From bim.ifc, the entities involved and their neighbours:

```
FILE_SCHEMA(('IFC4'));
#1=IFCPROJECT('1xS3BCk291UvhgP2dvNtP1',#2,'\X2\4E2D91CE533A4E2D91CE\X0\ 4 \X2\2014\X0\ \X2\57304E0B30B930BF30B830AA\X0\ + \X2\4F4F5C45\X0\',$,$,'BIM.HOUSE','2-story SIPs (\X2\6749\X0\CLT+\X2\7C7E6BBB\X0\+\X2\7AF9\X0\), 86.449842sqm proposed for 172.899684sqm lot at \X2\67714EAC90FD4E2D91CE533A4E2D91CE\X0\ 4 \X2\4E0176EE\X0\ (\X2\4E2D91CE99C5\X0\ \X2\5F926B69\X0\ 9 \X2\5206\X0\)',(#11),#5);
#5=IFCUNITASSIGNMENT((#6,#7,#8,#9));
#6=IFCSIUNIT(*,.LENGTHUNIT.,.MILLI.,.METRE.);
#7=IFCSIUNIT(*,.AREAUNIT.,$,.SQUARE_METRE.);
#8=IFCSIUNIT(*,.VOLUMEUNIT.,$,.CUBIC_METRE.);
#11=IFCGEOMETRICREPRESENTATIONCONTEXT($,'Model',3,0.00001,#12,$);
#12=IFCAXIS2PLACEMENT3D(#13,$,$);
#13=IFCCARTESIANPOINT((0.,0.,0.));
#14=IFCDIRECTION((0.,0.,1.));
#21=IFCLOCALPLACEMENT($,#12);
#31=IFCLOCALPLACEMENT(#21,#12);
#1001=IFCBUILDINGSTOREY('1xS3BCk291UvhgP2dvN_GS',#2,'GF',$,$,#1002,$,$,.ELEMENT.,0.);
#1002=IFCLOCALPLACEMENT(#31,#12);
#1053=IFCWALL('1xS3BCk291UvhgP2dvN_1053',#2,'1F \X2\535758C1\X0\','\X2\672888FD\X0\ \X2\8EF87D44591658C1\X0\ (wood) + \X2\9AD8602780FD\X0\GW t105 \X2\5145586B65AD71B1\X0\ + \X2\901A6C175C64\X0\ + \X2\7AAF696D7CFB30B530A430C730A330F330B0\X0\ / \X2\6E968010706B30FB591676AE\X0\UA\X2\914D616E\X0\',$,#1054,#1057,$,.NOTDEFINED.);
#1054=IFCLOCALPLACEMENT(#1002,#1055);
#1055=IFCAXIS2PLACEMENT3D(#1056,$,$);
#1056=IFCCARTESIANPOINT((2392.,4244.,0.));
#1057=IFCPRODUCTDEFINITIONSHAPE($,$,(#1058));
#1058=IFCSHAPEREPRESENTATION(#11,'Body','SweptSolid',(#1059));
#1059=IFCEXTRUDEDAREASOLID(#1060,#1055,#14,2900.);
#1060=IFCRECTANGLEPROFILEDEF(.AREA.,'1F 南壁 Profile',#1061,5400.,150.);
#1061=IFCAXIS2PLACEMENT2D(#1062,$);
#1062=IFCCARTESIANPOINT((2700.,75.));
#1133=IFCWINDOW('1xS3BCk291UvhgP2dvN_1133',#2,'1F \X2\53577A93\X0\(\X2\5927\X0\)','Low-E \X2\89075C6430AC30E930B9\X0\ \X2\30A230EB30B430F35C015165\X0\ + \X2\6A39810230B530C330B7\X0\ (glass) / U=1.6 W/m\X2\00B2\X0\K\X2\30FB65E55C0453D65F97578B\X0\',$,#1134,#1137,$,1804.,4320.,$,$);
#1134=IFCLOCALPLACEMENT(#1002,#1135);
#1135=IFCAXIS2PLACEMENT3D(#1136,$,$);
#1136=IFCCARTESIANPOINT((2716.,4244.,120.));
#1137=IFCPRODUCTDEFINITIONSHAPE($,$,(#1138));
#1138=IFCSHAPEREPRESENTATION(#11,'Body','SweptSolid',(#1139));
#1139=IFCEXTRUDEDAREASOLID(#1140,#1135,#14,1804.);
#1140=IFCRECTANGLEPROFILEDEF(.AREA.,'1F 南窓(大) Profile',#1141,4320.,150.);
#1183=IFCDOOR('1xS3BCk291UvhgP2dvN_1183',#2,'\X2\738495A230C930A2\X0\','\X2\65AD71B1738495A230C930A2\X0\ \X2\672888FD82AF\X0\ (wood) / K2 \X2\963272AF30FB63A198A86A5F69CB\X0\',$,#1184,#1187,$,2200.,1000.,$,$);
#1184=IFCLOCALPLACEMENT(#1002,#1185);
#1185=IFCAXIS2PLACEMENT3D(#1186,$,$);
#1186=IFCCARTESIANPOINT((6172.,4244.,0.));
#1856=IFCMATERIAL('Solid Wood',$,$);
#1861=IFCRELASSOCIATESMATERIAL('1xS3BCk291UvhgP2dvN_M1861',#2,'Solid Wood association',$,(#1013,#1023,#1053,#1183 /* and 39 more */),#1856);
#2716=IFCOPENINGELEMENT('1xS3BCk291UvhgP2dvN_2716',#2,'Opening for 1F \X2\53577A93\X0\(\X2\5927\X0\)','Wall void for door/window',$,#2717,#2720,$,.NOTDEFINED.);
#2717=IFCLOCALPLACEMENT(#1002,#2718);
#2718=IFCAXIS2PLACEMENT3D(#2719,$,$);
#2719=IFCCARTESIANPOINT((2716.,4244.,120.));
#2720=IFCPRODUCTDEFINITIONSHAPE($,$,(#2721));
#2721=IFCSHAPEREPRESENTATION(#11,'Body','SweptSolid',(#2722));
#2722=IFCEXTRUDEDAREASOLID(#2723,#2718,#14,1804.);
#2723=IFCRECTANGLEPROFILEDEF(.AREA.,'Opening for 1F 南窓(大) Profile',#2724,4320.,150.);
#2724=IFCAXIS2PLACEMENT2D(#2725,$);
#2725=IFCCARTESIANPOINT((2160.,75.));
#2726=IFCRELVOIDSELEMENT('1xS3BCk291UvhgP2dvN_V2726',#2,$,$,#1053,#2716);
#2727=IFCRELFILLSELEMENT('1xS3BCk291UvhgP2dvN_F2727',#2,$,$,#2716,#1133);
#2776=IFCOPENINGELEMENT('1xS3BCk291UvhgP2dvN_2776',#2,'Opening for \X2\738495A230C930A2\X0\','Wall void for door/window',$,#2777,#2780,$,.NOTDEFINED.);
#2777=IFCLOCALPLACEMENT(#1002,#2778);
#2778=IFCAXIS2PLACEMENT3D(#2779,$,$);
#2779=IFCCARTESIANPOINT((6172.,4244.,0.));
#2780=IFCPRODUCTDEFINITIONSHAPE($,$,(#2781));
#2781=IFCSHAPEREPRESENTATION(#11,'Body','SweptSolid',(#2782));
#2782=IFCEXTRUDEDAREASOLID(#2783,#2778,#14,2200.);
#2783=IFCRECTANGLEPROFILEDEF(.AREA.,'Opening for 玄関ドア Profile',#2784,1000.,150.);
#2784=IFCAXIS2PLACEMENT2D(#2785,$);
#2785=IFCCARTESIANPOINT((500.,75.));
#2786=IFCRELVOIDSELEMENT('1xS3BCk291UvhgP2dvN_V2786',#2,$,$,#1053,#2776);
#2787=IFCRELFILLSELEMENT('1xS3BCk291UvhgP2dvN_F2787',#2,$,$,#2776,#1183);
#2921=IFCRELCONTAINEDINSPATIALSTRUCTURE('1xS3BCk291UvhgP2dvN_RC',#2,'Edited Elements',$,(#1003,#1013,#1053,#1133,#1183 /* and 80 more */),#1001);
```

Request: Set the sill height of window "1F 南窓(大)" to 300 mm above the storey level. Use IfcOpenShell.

```python
import numpy as np
import ifcopenshell
import ifcopenshell.api.geometry
import ifcopenshell.geom
import ifcopenshell.util.element
import ifcopenshell.util.placement
import ifcopenshell.util.shape
import ifcopenshell.util.unit

model = ifcopenshell.open("bim.ifc")
unit_scale = ifcopenshell.util.unit.calculate_unit_scale(model)

window = model.by_id(1133)
opening = window.FillsVoids[0].RelatingOpeningElement
storey = ifcopenshell.util.element.get_container(window, ifc_class="IfcBuildingStorey")
level = ifcopenshell.util.placement.get_local_placement(storey.ObjectPlacement)[2, 3]

# The opening's origin need not be at the sill, so measure its lowest point.
shape = ifcopenshell.geom.create_shape(ifcopenshell.geom.settings(), opening)
bottom = ifcopenshell.util.shape.get_shape_bottom_elevation(shape, shape.geometry) / unit_scale
dz = level + 300.0 - bottom

shift = np.array([0.0, 0.0, dz])
# The window is not placed relative to its opening, so move both.
for product in (opening, window):
    matrix = ifcopenshell.util.placement.get_local_placement(product.ObjectPlacement)
    matrix[:3, 3] += shift
    ifcopenshell.api.geometry.edit_object_placement(model, product=product, matrix=matrix, is_si=False)

print(f"moved by {dz * unit_scale:+.3f} m")

model.write("bim_edited.ifc")
```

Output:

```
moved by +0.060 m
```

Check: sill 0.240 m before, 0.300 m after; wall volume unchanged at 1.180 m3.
